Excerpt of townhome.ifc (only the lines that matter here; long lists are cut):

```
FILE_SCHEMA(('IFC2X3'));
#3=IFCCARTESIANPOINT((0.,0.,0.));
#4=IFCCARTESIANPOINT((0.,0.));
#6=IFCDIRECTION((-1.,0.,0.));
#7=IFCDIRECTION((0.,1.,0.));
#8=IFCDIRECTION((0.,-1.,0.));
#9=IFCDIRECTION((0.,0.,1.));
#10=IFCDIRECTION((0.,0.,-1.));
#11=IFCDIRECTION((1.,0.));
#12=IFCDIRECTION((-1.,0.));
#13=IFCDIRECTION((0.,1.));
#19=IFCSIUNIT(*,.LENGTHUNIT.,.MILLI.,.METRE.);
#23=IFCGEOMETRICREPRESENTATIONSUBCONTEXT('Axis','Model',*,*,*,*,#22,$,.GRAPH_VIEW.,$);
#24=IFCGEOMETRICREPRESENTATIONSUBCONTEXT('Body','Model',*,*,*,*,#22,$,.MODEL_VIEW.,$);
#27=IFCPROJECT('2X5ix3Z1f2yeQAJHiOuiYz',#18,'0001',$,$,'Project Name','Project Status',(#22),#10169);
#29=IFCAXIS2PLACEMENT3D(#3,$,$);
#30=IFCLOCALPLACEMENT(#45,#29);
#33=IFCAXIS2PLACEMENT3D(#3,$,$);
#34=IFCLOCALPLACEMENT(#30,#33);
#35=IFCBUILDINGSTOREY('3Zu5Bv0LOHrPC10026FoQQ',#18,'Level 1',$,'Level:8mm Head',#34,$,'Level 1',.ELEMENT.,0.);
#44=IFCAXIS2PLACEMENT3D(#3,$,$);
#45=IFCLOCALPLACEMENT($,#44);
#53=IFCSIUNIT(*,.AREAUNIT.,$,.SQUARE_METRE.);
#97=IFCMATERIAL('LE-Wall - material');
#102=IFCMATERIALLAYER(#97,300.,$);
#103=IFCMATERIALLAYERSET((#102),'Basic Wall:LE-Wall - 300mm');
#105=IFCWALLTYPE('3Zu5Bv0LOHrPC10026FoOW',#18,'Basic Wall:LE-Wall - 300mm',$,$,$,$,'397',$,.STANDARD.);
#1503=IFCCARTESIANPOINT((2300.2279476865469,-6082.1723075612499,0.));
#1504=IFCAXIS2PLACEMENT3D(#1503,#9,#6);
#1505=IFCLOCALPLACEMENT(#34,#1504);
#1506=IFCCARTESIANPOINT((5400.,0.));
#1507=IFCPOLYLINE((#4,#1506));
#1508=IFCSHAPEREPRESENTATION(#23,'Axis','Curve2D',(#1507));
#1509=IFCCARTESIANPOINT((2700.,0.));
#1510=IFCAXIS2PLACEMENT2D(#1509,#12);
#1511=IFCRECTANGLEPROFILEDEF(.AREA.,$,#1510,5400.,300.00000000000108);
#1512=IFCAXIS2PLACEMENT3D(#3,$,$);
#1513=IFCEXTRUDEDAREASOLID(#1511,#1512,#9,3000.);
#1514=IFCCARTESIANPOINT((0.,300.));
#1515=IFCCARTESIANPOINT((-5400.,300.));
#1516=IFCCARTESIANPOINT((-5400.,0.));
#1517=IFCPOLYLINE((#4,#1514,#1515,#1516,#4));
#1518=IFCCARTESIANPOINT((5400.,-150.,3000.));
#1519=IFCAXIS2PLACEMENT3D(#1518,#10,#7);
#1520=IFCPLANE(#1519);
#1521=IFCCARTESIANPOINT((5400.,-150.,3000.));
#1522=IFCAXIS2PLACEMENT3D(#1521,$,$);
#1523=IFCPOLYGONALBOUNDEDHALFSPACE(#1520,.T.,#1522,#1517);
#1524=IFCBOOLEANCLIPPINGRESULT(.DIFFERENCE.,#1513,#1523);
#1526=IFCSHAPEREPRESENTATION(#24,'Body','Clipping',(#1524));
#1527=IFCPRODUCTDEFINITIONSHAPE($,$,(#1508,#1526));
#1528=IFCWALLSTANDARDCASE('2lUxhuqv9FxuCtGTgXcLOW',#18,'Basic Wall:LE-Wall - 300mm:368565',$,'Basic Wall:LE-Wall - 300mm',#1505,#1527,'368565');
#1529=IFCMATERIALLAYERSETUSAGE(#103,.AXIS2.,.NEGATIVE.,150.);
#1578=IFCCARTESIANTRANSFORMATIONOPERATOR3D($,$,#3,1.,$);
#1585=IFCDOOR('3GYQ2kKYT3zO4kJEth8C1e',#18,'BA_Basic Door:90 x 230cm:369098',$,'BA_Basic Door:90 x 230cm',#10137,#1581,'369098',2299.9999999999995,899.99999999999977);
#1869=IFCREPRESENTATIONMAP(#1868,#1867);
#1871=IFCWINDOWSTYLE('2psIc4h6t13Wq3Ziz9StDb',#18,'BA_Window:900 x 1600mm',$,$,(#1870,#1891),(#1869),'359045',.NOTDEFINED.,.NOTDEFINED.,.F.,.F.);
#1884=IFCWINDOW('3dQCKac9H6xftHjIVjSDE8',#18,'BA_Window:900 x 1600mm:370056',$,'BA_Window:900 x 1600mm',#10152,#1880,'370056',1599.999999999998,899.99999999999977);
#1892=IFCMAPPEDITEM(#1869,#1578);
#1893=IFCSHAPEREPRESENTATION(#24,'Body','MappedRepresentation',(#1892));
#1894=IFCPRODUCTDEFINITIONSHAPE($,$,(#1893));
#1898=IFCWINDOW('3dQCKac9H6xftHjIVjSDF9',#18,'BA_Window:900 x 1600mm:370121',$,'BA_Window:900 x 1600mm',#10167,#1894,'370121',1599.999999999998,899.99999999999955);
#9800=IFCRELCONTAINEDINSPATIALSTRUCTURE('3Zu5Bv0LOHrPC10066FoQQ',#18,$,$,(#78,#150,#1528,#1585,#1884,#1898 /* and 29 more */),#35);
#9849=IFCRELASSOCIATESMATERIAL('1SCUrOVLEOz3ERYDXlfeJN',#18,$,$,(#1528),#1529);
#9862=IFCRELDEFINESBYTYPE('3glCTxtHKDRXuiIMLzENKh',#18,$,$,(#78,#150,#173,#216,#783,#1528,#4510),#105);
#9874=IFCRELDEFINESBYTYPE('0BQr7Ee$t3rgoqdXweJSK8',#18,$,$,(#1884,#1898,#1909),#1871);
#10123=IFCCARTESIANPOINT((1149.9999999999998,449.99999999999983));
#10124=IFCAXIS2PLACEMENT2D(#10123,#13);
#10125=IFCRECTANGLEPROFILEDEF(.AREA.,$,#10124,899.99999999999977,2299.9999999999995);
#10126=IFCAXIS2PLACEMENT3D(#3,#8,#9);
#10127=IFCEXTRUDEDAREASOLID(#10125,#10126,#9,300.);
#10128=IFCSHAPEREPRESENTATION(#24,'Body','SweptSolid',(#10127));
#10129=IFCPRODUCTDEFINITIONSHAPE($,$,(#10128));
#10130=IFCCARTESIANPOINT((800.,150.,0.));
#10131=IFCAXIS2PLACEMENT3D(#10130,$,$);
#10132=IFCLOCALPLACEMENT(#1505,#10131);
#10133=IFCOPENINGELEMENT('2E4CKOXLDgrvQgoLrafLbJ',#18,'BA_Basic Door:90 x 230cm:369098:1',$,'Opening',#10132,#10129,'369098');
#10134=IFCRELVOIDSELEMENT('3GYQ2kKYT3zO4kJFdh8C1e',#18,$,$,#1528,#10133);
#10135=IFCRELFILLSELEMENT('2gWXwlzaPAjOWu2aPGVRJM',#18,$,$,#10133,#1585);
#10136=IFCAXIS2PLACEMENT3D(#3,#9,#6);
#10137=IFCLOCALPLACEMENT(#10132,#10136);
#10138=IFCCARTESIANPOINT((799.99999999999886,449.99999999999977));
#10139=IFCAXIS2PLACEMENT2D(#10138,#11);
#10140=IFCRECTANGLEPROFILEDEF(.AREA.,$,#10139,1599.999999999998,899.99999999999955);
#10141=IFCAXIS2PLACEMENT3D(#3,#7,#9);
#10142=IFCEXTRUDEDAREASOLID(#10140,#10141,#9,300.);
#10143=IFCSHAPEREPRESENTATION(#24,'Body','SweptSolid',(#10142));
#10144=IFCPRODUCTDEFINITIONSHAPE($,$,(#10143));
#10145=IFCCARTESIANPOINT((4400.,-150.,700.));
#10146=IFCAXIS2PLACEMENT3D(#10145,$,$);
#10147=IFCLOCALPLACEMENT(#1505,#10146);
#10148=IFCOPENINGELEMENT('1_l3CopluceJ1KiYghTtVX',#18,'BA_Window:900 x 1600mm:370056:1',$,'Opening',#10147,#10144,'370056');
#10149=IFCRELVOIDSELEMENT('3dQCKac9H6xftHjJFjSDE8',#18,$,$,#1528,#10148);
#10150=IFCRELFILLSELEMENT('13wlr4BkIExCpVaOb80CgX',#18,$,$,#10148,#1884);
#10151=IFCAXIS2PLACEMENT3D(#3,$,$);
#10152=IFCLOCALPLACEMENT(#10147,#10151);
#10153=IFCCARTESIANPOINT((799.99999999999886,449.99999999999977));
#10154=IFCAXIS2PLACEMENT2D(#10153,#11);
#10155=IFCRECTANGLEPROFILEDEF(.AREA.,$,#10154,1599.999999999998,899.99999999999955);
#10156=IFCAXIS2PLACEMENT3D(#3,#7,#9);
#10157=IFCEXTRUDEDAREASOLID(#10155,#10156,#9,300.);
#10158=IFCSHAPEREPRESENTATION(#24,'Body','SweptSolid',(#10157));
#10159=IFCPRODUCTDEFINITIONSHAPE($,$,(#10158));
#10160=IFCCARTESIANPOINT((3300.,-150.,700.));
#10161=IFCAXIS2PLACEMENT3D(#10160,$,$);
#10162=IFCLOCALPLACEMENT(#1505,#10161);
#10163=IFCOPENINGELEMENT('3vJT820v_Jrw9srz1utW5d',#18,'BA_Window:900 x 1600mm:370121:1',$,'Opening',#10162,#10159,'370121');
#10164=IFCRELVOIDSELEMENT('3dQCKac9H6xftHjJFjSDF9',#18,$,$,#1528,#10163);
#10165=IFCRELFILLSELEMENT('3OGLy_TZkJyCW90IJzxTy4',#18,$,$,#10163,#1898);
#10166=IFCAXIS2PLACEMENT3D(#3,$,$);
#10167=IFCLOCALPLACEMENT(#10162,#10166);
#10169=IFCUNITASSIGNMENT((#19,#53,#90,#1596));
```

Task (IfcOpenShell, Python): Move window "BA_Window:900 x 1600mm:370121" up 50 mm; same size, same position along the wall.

```python
import numpy as np
import ifcopenshell
import ifcopenshell.api.geometry
import ifcopenshell.util.placement
import ifcopenshell.util.unit

model = ifcopenshell.open("townhome.ifc")
unit_scale = ifcopenshell.util.unit.calculate_unit_scale(model)

window = model.by_guid("3dQCKac9H6xftHjIVjSDF9")
opening = window.FillsVoids[0].RelatingOpeningElement
dz = 0.05 / unit_scale

shift = np.array([0.0, 0.0, dz])
# The window is placed relative to its opening, so it follows when the opening moves.
matrix = ifcopenshell.util.placement.get_local_placement(opening.ObjectPlacement)
matrix[:3, 3] += shift
ifcopenshell.api.geometry.edit_object_placement(
    model, product=opening, matrix=matrix, is_si=False, should_transform_children=True
)

print(f"moved by {dz * unit_scale:+.3f} m")

model.write("townhome_rev.ifc")
```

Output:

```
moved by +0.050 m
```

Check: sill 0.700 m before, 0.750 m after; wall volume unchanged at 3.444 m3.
